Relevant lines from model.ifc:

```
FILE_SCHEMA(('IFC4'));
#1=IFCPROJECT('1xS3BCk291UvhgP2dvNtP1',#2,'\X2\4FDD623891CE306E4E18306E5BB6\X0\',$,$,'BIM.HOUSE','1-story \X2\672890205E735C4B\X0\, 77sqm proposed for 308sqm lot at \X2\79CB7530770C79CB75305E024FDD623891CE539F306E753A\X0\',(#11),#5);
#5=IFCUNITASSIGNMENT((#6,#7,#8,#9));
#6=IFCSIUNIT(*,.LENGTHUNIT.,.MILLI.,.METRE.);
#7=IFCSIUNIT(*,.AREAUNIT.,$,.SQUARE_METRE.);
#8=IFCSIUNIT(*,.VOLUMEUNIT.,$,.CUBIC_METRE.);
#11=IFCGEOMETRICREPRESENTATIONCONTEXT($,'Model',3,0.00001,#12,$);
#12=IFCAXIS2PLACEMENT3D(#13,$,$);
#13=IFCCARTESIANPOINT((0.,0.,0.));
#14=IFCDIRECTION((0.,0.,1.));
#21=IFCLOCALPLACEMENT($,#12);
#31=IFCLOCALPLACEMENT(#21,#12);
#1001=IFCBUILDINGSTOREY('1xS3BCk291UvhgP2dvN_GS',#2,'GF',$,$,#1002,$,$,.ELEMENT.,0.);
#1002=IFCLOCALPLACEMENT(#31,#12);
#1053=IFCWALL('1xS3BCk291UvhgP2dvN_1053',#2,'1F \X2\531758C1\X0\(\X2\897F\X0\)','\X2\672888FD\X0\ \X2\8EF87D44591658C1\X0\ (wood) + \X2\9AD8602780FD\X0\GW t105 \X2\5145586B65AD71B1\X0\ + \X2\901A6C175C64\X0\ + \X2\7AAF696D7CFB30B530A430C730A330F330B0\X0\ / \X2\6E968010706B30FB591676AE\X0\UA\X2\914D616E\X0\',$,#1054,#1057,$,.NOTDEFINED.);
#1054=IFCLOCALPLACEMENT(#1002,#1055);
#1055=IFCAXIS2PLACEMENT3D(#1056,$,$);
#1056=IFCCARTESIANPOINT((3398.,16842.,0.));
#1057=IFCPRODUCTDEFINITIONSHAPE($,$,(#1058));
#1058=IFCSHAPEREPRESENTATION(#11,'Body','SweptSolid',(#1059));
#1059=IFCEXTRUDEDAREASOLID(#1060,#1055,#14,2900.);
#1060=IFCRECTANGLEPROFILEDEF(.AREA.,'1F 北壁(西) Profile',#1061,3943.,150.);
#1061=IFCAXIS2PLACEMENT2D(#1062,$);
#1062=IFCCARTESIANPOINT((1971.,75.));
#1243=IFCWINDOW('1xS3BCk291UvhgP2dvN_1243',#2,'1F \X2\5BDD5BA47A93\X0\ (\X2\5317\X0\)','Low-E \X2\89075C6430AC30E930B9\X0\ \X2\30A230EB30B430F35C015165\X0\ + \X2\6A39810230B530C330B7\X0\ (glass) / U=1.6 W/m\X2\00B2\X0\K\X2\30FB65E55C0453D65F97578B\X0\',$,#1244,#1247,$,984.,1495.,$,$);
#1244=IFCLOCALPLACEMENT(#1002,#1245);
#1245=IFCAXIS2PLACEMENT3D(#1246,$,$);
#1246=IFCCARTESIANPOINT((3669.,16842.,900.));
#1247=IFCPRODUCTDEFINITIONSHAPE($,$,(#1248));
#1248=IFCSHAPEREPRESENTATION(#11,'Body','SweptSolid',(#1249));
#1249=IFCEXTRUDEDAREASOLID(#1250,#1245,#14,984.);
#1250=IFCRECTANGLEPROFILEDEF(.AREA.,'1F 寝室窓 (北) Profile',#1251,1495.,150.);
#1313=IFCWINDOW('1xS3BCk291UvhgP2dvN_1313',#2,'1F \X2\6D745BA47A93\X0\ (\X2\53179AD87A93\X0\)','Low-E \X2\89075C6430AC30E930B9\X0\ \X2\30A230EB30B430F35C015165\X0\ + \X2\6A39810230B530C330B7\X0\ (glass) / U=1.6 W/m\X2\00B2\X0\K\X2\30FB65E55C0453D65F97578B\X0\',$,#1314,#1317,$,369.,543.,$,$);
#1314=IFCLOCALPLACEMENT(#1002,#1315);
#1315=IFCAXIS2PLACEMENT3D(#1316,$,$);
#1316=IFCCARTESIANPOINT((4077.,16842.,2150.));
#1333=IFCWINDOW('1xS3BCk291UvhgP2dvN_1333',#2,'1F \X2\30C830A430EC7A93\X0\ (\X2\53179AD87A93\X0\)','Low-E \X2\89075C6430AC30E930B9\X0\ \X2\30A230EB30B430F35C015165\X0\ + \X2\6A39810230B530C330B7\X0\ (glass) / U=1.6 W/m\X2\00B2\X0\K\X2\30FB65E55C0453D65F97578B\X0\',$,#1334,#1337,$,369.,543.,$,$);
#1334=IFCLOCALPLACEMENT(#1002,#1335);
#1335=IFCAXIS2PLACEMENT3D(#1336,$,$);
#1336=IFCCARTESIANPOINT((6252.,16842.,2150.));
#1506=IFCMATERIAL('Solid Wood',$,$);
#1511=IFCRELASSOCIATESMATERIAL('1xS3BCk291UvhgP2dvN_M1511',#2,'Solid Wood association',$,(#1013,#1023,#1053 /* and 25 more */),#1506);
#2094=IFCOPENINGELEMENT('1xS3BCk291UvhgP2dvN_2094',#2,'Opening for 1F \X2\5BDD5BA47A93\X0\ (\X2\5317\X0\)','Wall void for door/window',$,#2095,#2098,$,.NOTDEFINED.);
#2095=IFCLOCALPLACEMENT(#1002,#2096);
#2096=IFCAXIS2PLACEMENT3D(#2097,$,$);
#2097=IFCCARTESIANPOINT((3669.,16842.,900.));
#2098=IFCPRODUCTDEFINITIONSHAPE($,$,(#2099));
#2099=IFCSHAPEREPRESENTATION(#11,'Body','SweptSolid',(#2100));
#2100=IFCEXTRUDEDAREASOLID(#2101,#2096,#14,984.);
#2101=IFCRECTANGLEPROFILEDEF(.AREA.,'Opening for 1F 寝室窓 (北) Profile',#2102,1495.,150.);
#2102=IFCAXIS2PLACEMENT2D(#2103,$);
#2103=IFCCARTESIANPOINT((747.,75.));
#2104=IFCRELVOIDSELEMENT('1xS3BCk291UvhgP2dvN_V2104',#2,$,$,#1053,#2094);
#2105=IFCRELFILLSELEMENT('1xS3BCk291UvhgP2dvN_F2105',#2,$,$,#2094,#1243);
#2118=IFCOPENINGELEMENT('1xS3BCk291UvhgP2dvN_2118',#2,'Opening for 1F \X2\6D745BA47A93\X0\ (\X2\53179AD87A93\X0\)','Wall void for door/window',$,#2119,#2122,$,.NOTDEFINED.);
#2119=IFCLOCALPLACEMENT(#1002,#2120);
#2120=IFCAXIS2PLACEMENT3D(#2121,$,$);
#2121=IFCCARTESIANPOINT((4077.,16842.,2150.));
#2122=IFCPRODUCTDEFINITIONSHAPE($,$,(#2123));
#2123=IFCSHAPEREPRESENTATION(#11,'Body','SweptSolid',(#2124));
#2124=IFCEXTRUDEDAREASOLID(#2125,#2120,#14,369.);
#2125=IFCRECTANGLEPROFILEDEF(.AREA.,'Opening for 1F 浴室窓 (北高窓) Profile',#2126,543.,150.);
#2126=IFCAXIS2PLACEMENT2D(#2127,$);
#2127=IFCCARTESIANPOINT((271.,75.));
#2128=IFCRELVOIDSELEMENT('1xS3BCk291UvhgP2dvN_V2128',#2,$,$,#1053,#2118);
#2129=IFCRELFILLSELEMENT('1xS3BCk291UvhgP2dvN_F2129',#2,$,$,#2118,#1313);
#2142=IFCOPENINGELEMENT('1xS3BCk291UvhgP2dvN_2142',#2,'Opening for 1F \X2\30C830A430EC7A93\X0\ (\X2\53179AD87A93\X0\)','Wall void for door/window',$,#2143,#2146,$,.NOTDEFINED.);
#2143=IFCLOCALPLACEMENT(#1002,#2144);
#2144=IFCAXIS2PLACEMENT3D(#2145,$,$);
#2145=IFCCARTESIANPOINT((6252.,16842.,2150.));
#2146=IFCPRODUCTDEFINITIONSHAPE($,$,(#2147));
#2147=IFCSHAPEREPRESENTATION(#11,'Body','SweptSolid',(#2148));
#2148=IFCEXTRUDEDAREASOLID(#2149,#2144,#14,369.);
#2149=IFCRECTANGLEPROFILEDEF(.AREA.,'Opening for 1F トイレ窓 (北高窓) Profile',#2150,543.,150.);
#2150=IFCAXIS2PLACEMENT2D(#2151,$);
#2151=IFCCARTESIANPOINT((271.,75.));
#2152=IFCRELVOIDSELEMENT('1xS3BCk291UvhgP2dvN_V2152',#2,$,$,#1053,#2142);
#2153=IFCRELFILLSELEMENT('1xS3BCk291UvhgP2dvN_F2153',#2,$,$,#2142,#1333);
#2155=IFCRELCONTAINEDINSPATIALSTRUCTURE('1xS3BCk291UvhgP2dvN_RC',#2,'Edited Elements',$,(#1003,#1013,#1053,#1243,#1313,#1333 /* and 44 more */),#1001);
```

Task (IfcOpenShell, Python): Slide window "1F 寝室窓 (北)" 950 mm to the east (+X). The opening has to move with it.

```python
import ifcopenshell
import ifcopenshell.api.geometry
import ifcopenshell.util.placement
import ifcopenshell.util.unit

model = ifcopenshell.open("model.ifc")
unit_scale = ifcopenshell.util.unit.calculate_unit_scale(model)

window = model.by_guid("1xS3BCk291UvhgP2dvN_1243")
opening = window.FillsVoids[0].RelatingOpeningElement
wall = opening.VoidsElements[0].RelatingBuildingElement

wall_matrix = ifcopenshell.util.placement.get_local_placement(wall.ObjectPlacement)
shift = wall_matrix[:3, 0] * 0.95 / unit_scale
before = ifcopenshell.util.placement.get_local_placement(window.ObjectPlacement)[:3, 3].copy()

# The window is not placed relative to its opening, so move both.
for product in (opening, window):
    matrix = ifcopenshell.util.placement.get_local_placement(product.ObjectPlacement)
    matrix[:3, 3] += shift
    ifcopenshell.api.geometry.edit_object_placement(model, product=product, matrix=matrix, is_si=False)

after = ifcopenshell.util.placement.get_local_placement(window.ObjectPlacement)[:3, 3]
print("window moved by", (after - before).round(3) + 0.0)

model.write("model_updated.ifc")
```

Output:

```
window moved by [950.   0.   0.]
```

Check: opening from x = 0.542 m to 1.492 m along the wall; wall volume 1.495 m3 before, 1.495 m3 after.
